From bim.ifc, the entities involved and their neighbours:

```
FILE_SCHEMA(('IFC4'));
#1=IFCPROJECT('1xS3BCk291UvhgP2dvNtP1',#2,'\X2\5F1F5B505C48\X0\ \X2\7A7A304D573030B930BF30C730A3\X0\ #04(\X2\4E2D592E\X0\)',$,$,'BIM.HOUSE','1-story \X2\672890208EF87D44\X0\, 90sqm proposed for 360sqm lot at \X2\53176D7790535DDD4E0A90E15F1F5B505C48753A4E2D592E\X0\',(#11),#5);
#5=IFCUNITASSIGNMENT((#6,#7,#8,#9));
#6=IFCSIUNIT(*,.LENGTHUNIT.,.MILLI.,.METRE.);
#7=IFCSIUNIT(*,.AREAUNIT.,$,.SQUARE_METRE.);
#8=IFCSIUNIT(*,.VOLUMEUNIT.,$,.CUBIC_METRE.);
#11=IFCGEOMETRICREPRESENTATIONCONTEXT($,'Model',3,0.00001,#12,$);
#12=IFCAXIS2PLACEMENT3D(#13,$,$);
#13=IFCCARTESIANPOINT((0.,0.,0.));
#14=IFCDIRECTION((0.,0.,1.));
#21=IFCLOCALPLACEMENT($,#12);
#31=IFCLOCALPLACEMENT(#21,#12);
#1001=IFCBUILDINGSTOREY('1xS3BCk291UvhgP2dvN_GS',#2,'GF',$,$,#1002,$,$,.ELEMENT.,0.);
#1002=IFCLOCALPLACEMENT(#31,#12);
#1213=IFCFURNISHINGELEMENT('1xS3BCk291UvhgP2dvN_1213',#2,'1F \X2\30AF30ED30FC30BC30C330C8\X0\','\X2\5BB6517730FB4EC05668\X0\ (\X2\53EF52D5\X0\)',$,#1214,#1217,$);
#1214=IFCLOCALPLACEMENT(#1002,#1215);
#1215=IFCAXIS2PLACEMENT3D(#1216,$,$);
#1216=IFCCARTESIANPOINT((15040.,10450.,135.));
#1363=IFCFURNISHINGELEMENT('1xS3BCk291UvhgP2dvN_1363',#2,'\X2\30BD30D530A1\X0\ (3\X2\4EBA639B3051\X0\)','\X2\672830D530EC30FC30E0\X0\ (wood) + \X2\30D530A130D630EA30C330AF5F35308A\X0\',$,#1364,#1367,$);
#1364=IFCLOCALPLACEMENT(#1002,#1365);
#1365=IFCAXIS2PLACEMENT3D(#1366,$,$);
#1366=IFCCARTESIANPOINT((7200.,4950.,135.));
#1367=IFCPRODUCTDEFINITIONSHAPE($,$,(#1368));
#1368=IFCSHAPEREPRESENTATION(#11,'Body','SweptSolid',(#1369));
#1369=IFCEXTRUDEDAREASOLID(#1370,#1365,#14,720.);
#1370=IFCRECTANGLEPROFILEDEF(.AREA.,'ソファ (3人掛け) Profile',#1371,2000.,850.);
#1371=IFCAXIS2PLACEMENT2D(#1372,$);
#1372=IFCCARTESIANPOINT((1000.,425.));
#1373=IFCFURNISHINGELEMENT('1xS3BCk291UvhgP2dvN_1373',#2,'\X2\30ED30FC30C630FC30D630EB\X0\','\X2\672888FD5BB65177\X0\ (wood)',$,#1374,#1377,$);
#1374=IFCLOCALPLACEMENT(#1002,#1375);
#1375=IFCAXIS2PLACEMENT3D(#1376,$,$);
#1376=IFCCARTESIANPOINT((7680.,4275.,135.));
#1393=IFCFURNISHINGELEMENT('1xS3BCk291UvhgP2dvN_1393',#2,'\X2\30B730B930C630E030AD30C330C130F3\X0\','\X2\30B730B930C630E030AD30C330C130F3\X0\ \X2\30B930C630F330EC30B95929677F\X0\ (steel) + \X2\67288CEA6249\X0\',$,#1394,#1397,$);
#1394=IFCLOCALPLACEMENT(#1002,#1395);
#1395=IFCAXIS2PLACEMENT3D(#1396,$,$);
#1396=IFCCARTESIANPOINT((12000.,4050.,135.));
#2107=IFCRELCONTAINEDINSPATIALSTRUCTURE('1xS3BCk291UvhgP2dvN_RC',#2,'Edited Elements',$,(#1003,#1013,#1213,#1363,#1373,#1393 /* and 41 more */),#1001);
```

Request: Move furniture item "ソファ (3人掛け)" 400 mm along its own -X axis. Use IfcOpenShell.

```python
import ifcopenshell
import ifcopenshell.api.geometry
import ifcopenshell.util.placement

model = ifcopenshell.open("bim.ifc")

item = model.by_id(1363)
matrix = ifcopenshell.util.placement.get_local_placement(item.ObjectPlacement)
matrix[:3, 3] -= matrix[:3, 0] * 400.0
ifcopenshell.api.geometry.edit_object_placement(model, product=item, matrix=matrix, is_si=False)

print(ifcopenshell.util.placement.get_local_placement(item.ObjectPlacement).round(3) + 0.0)

model.write("bim_v2.ifc")
```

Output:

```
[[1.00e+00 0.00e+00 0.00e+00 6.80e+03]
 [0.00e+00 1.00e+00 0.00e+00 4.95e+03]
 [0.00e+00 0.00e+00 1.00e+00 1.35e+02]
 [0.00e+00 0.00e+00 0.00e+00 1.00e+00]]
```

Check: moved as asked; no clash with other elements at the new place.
